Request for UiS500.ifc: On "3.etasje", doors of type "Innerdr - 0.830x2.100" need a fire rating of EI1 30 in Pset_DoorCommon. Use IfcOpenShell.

First a look at what the model holds.

```python
import ifcopenshell
import ifcopenshell.util.element

model = ifcopenshell.open("UiS500.ifc")
print(model.schema)
storey = next(s for s in model.by_type("IfcBuildingStorey") if s.Name == "3.etasje")
doors = [e for e in ifcopenshell.util.element.get_decomposition(storey) if e.is_a("IfcDoor")]
seen = {}
for e in doors:
    element_type = ifcopenshell.util.element.get_type(e)
    key = (element_type.Name if element_type != e and element_type else None, ifcopenshell.util.element.get_pset(e, "Pset_DoorCommon", "FireRating"))
    seen[key] = seen.get(key, 0) + 1
for (name, value), count in sorted(seen.items(), key=str):
    print(count, "x", name, "|", value)
```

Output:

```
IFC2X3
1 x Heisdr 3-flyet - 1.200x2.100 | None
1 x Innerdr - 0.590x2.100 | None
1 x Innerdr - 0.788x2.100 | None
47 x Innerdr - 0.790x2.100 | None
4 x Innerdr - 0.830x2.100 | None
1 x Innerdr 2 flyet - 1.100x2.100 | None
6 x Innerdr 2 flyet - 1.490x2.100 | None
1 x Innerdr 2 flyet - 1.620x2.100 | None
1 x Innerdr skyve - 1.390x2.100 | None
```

```python
import ifcopenshell
import ifcopenshell.api.pset
import ifcopenshell.util.element

model = ifcopenshell.open("UiS500.ifc")

storey = next(s for s in model.by_type("IfcBuildingStorey") if s.Name == "3.etasje")
doors = [e for e in ifcopenshell.util.element.get_decomposition(storey) if e.is_a("IfcDoor")]

count = 0
for e in doors:
    element_type = ifcopenshell.util.element.get_type(e)
    if element_type in (None, e) or element_type.Name != 'Innerd\x9br - 0.830x2.100':
        continue
    # add_pset returns the element's existing set when there is one.
    pset = ifcopenshell.api.pset.add_pset(model, product=e, name="Pset_DoorCommon")
    ifcopenshell.api.pset.edit_pset(model, pset=pset, properties={"FireRating": "EI1 30"})
    count += 1

print(count, "doors updated")

model.write("UiS500_rev.ifc")
```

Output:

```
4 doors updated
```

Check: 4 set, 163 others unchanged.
